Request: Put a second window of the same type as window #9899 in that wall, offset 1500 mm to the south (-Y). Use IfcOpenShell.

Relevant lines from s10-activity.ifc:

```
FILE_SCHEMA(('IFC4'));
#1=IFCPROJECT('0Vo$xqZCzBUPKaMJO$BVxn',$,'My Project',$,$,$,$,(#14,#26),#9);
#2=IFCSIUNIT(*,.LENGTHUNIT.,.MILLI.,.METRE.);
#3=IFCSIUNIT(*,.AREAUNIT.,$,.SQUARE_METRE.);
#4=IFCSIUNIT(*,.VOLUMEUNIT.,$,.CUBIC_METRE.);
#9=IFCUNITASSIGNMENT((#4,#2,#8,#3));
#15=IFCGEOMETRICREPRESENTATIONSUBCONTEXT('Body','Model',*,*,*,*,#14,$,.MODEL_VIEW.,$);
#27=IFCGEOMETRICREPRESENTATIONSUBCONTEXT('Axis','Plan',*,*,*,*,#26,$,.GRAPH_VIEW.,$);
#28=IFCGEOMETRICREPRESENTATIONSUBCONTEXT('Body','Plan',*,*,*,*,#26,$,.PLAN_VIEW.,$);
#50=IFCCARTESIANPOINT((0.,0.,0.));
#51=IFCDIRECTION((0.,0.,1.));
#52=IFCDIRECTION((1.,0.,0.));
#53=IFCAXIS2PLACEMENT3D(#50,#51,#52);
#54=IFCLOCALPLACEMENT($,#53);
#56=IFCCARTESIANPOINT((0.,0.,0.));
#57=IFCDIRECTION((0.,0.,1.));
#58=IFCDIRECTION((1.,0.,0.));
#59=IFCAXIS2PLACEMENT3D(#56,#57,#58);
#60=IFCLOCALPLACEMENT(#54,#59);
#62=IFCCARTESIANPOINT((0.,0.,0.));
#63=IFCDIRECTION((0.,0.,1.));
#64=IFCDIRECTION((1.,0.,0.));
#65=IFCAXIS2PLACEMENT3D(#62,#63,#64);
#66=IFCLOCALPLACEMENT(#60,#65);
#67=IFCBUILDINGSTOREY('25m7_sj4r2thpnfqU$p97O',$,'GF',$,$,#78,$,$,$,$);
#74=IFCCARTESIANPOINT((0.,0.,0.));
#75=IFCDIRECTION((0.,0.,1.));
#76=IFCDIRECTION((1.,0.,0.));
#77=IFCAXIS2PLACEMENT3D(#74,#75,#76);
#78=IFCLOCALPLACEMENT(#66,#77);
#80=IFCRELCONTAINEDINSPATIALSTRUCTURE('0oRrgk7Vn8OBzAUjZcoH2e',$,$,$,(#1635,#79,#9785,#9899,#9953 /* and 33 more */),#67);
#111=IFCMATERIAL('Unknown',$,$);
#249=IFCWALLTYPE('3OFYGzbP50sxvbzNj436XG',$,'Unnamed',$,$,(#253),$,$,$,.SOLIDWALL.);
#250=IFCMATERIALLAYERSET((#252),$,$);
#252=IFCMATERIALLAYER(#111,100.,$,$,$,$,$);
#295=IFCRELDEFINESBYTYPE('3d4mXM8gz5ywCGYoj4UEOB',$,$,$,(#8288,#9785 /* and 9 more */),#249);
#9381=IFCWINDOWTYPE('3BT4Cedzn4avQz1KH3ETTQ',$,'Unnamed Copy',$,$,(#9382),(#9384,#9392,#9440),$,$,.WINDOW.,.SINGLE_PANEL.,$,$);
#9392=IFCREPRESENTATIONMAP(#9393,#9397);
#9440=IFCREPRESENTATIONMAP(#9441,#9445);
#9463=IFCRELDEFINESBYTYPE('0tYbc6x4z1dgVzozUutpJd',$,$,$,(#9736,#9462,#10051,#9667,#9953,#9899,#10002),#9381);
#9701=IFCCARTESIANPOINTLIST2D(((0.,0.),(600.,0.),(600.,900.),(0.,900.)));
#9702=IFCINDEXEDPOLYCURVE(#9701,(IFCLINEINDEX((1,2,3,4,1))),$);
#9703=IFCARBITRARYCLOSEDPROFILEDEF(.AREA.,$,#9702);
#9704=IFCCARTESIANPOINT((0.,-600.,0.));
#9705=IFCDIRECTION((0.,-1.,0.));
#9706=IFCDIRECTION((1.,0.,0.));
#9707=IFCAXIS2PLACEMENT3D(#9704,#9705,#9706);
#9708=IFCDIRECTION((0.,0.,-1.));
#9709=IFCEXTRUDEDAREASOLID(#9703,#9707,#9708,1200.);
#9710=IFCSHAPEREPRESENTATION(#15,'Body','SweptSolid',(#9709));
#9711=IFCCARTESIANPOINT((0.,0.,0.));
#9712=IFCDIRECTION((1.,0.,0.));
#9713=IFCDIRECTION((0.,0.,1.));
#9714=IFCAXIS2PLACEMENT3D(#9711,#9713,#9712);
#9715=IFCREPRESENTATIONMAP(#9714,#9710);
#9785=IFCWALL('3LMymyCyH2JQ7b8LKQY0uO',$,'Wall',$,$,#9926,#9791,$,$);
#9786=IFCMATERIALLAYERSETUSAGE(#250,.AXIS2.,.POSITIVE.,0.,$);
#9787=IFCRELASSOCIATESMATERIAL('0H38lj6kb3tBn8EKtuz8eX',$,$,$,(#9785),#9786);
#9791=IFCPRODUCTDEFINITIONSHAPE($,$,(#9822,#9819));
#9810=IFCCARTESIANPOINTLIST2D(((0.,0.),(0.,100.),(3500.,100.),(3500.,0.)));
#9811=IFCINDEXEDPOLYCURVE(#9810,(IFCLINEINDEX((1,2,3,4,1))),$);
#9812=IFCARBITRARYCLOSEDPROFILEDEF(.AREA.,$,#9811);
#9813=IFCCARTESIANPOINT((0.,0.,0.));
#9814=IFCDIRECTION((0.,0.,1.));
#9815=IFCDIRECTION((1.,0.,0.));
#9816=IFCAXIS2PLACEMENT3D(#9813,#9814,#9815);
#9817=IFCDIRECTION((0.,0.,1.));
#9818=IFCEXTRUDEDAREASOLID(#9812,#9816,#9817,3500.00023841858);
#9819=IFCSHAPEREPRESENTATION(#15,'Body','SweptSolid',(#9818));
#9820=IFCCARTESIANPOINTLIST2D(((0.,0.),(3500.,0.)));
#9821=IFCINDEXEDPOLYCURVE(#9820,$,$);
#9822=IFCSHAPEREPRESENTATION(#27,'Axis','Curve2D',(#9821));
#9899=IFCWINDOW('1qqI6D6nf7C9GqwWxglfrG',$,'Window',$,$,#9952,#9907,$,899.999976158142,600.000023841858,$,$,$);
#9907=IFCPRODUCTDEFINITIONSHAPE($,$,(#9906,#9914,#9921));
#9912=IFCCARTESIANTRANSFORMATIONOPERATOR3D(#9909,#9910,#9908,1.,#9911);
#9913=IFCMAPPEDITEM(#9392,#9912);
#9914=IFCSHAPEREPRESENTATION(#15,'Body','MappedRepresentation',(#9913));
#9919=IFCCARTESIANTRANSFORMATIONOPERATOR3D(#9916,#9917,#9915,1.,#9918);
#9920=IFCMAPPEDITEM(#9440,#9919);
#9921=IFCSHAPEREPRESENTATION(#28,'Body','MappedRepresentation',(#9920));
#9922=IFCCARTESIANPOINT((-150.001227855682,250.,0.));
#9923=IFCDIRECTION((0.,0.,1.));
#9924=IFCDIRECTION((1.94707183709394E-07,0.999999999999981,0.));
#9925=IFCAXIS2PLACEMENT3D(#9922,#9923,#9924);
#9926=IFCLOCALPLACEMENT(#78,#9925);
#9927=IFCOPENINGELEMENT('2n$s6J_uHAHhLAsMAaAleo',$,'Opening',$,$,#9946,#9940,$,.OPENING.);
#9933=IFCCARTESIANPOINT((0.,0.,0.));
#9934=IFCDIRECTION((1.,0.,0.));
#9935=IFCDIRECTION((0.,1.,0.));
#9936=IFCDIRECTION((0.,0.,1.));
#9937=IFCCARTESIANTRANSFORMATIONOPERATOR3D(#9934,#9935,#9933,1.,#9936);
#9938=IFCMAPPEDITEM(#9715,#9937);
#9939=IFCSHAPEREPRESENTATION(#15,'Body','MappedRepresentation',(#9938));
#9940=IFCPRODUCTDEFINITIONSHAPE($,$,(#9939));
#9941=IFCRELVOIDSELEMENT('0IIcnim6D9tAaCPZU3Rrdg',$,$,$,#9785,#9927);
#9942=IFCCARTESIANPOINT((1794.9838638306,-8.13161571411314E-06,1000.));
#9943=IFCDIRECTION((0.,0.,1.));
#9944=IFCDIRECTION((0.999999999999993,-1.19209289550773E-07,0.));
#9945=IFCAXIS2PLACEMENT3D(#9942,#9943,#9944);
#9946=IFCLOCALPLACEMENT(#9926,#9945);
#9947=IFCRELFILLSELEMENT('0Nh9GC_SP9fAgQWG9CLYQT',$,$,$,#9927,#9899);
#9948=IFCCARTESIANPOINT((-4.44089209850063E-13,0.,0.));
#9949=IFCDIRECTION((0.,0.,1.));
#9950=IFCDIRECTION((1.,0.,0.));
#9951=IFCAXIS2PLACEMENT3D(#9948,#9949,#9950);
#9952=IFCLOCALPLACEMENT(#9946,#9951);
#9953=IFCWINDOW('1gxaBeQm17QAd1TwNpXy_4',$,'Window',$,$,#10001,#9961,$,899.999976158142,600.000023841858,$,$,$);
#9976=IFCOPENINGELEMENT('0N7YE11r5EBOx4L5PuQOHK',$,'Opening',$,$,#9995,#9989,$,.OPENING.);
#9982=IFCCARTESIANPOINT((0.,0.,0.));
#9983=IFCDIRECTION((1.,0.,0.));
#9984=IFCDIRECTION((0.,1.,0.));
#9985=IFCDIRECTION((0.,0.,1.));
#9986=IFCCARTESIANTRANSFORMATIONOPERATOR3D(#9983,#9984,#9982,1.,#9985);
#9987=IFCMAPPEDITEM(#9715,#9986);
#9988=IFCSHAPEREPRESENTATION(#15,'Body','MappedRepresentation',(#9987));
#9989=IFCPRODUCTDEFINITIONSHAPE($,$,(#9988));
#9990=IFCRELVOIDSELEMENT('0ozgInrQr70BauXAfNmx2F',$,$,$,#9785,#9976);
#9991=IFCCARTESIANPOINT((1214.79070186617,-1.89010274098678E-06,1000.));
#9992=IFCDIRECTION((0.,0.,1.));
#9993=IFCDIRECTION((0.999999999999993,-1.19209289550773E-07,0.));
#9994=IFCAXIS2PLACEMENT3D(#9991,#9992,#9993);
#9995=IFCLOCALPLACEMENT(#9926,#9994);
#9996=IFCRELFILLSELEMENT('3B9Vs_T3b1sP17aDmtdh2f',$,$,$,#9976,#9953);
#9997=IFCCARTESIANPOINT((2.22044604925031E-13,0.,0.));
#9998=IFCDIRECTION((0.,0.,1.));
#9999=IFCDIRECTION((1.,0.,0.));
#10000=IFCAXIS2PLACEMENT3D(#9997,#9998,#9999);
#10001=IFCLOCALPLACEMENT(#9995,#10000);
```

```python
import ifcopenshell
import ifcopenshell.api.feature
import ifcopenshell.api.geometry
import ifcopenshell.api.root
import ifcopenshell.geom
import ifcopenshell.util.element
import ifcopenshell.util.placement
import ifcopenshell.util.shape
import ifcopenshell.util.unit

model = ifcopenshell.open("s10-activity.ifc")
unit_scale = ifcopenshell.util.unit.calculate_unit_scale(model)
settings = ifcopenshell.geom.settings()


def volume(element):
    """Net volume in cubic metres, openings subtracted."""
    shape = ifcopenshell.geom.create_shape(settings, element)
    return ifcopenshell.util.shape.get_volume(shape.geometry)


window = model.by_id(9899)
opening = window.FillsVoids[0].RelatingOpeningElement
wall = opening.VoidsElements[0].RelatingBuildingElement
before = volume(wall)
shift = ifcopenshell.util.placement.get_local_placement(wall.ObjectPlacement)[:3, 0] * -1.5 / unit_scale

# copy_class copies the void relationship, type, container and properties, but no geometry.
new_opening = ifcopenshell.api.root.copy_class(model, product=opening)
new_opening.Representation = ifcopenshell.util.element.copy_deep(
    model, opening.Representation, exclude=["IfcGeometricRepresentationContext", "IfcRepresentationMap"]
)
new_window = ifcopenshell.api.root.copy_class(model, product=window)
new_window.Representation = ifcopenshell.util.element.copy_deep(
    model, window.Representation, exclude=["IfcGeometricRepresentationContext", "IfcRepresentationMap"]
)
ifcopenshell.api.feature.add_filling(model, opening=new_opening, element=new_window)

for old, new in ((opening, new_opening), (window, new_window)):
    matrix = ifcopenshell.util.placement.get_local_placement(old.ObjectPlacement)
    matrix[:3, 3] += shift
    ifcopenshell.api.geometry.edit_object_placement(model, product=new, matrix=matrix, is_si=False)

after = volume(wall)

print(f"wall volume {before:.3f} -> {after:.3f} m3")

model.write("s10-activity_v2.ifc")
```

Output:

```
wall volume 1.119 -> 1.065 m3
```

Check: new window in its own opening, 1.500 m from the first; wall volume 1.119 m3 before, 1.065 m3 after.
